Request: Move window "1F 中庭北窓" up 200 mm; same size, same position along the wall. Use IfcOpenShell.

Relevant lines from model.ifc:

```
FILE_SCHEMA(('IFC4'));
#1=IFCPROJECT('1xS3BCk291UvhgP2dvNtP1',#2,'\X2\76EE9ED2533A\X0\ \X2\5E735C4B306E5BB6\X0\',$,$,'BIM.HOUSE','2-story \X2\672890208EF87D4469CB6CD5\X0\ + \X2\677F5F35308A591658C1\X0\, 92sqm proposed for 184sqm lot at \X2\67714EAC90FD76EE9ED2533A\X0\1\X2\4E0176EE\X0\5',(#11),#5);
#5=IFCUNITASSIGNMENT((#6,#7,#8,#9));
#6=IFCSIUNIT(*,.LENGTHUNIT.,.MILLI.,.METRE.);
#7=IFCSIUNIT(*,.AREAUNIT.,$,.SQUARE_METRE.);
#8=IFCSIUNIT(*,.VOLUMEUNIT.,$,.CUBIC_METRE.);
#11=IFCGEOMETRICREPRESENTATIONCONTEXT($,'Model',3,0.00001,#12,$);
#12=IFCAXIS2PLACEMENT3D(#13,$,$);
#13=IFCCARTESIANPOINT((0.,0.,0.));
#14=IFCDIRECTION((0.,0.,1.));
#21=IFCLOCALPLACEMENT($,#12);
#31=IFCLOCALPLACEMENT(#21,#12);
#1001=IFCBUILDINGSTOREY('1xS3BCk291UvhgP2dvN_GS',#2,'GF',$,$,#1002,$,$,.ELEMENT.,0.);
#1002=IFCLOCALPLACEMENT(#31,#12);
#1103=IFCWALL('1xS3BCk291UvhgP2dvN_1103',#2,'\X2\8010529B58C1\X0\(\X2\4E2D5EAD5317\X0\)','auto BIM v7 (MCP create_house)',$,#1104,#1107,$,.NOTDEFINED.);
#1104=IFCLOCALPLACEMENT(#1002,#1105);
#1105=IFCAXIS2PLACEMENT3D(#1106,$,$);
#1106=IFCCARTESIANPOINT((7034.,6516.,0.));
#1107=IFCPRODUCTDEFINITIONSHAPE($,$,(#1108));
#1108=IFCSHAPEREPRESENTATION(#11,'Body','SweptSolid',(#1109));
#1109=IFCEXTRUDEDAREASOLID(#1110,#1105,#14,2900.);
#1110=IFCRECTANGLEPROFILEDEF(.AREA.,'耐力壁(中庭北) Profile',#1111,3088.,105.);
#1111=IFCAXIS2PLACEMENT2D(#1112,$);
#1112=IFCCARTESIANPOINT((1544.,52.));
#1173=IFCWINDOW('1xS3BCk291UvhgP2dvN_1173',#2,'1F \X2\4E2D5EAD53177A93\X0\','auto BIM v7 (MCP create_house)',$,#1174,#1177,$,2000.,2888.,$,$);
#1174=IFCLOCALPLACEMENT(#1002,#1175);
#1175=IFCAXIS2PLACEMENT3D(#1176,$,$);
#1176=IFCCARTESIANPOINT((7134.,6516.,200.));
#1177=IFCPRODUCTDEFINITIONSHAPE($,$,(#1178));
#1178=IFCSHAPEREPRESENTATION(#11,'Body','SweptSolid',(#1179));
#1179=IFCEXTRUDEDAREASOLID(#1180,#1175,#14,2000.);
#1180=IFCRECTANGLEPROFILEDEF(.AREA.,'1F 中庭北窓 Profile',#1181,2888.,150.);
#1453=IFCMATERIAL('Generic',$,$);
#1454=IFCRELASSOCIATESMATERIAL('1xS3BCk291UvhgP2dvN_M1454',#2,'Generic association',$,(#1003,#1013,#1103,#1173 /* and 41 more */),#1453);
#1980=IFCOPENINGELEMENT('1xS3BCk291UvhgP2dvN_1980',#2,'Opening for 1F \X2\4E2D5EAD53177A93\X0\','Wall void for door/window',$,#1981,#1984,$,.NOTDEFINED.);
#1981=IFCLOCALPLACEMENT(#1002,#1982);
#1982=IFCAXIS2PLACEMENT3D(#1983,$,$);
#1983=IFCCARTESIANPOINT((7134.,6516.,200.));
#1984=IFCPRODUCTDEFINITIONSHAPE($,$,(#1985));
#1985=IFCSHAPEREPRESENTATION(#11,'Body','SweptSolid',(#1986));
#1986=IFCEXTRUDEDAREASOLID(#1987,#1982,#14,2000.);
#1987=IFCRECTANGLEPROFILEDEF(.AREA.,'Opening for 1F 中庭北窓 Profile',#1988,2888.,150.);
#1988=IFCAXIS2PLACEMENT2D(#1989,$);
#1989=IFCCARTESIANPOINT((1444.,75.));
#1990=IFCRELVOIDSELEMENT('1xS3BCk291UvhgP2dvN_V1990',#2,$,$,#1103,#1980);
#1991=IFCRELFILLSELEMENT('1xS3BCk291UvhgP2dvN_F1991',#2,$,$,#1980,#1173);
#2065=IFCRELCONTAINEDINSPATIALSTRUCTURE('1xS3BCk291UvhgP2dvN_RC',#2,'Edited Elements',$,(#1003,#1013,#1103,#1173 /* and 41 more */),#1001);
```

```python
import numpy as np
import ifcopenshell
import ifcopenshell.api.geometry
import ifcopenshell.util.placement
import ifcopenshell.util.unit

model = ifcopenshell.open("model.ifc")
unit_scale = ifcopenshell.util.unit.calculate_unit_scale(model)

window = model.by_guid("1xS3BCk291UvhgP2dvN_1173")
opening = window.FillsVoids[0].RelatingOpeningElement
dz = 200.0

shift = np.array([0.0, 0.0, dz])
# The window is not placed relative to its opening, so move both.
for product in (opening, window):
    matrix = ifcopenshell.util.placement.get_local_placement(product.ObjectPlacement)
    matrix[:3, 3] += shift
    ifcopenshell.api.geometry.edit_object_placement(model, product=product, matrix=matrix, is_si=False)

print(f"moved by {dz * unit_scale:+.3f} m")

model.write("model_updated.ifc")
```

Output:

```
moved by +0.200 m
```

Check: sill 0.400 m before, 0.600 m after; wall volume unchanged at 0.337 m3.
